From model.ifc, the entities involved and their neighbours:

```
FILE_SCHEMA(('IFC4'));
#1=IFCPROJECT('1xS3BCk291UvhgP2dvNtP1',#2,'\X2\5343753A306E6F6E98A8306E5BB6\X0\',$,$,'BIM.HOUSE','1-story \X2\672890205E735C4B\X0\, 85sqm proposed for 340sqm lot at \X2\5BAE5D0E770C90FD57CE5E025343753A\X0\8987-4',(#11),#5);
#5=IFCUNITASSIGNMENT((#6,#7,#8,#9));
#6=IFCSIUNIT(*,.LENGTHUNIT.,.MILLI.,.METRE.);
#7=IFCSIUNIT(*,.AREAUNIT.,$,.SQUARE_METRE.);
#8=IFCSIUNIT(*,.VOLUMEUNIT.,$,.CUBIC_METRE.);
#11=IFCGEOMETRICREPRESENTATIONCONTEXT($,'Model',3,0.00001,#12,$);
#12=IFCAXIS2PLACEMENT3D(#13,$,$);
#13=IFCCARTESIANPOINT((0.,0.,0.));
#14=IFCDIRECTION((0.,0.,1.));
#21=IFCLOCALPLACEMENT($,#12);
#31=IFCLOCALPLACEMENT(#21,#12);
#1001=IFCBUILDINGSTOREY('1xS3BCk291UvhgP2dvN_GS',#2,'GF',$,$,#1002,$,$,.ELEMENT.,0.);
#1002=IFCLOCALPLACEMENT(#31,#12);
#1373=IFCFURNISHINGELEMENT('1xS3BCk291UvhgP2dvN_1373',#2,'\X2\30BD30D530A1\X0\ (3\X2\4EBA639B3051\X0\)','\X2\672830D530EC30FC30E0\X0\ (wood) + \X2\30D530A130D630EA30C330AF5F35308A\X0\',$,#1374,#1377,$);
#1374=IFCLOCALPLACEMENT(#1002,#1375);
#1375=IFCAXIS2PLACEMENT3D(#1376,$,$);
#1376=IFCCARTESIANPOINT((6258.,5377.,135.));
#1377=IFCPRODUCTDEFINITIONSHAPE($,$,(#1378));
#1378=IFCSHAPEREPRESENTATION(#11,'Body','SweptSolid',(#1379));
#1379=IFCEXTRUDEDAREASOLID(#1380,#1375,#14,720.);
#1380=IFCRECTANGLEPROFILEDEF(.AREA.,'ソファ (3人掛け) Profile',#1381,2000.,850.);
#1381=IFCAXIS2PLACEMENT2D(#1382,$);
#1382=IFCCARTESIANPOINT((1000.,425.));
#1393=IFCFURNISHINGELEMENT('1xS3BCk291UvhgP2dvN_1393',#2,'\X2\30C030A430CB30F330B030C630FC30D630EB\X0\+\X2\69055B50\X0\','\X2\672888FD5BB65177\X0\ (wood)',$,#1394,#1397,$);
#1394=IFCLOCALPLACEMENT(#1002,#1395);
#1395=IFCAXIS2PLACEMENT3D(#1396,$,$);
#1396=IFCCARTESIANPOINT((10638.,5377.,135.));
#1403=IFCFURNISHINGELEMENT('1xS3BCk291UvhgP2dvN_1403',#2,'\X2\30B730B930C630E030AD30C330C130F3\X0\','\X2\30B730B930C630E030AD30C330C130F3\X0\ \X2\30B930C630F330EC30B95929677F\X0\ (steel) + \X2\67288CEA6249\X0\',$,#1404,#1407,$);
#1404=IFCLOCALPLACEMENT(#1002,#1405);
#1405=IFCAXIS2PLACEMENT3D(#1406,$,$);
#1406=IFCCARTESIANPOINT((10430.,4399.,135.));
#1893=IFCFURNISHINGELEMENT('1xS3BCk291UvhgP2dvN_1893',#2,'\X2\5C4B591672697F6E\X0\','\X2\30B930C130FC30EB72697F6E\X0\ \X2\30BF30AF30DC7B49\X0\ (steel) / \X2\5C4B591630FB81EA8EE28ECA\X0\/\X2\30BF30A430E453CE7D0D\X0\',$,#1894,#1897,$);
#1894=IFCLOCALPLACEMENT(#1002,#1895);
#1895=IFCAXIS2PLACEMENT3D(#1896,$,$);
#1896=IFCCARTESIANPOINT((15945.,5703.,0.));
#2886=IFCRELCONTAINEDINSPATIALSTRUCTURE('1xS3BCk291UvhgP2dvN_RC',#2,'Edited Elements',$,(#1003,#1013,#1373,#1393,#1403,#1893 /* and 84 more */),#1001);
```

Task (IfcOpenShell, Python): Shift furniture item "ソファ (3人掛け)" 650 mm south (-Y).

```python
import ifcopenshell
import ifcopenshell.api.geometry
import ifcopenshell.util.placement
import ifcopenshell.util.unit

model = ifcopenshell.open("model.ifc")
unit_scale = ifcopenshell.util.unit.calculate_unit_scale(model)

item = model.by_guid("1xS3BCk291UvhgP2dvN_1373")
matrix = ifcopenshell.util.placement.get_local_placement(item.ObjectPlacement)
matrix[1, 3] -= 0.65 / unit_scale
ifcopenshell.api.geometry.edit_object_placement(model, product=item, matrix=matrix, is_si=False)

print(ifcopenshell.util.placement.get_local_placement(item.ObjectPlacement).round(3) + 0.0)

model.write("model_edited.ifc")
```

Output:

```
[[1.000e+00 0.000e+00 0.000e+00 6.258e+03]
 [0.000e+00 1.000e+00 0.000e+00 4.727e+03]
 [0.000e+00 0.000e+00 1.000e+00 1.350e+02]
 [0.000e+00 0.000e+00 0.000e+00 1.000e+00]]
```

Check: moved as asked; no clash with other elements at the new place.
